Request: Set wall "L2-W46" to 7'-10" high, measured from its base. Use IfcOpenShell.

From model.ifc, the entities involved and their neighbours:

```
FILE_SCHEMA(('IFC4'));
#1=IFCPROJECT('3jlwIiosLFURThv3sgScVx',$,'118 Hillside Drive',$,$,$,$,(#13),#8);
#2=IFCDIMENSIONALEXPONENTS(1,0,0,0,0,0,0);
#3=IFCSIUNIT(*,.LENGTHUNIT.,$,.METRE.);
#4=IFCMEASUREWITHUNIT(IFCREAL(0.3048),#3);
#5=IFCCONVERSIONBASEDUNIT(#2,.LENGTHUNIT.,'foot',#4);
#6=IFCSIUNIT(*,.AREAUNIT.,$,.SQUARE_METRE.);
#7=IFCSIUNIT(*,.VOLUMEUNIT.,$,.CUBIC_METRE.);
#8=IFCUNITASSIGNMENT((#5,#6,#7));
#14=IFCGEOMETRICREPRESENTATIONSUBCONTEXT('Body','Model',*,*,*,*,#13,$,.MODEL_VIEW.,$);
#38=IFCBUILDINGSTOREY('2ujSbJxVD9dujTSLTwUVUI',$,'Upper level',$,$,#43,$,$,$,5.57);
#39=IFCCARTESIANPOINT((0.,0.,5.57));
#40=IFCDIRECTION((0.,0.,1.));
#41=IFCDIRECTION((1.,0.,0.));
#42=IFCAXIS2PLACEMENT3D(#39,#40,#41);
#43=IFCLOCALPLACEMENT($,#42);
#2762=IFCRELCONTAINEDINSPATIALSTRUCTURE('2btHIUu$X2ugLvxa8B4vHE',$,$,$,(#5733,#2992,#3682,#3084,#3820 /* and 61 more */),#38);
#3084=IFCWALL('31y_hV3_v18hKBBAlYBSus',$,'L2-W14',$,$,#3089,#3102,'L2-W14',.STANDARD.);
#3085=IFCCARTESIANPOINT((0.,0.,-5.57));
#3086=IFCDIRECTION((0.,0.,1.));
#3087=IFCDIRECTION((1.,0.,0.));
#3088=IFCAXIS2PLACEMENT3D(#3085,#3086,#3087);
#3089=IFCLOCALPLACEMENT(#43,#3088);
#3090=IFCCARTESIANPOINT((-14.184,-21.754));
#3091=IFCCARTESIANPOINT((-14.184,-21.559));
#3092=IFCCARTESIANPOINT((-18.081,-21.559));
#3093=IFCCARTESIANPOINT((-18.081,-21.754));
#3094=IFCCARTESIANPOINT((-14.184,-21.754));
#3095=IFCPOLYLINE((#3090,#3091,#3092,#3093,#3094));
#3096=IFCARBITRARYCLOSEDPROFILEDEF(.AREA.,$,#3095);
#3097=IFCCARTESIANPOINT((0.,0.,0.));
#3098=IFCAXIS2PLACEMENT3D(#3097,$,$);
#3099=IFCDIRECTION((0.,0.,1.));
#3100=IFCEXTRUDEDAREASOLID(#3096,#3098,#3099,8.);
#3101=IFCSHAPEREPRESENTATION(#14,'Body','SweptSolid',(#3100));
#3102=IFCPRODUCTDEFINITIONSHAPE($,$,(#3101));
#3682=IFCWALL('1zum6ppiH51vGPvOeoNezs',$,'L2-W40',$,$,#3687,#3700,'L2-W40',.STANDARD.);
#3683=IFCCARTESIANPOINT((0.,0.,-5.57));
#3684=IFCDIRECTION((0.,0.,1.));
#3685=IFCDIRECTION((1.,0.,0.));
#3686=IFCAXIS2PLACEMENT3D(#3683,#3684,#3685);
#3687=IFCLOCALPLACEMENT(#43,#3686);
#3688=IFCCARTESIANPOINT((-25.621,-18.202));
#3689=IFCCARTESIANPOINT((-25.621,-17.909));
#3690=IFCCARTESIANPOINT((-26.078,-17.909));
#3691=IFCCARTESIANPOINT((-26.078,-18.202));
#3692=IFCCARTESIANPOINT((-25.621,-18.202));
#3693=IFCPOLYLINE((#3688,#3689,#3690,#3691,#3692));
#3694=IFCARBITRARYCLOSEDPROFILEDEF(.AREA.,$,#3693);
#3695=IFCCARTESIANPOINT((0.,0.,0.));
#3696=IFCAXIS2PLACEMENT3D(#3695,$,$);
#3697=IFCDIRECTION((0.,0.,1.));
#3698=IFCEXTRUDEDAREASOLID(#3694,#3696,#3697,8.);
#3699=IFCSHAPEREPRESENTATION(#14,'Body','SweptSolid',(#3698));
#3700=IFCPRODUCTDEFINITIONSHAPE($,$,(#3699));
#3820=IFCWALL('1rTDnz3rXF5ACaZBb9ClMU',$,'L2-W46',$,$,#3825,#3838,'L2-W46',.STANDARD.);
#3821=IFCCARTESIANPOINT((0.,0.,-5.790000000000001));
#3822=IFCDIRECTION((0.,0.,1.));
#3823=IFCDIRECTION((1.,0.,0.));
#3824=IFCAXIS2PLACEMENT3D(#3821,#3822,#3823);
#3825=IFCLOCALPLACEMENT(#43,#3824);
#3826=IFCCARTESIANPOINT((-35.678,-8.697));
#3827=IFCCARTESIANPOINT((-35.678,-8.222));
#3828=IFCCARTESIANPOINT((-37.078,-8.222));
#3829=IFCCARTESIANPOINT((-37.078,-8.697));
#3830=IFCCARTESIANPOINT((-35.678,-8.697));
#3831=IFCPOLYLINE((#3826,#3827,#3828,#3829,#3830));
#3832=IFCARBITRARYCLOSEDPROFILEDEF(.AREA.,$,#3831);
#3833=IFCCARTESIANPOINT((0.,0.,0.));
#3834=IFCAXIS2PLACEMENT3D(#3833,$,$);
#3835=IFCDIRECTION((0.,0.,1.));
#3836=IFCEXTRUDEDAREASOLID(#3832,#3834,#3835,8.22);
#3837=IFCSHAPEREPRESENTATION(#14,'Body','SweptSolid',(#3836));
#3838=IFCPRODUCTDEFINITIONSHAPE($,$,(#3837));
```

```python
import ifcopenshell
import ifcopenshell.geom
import ifcopenshell.util.representation
import ifcopenshell.util.shape
import ifcopenshell.util.unit

model = ifcopenshell.open("model.ifc")
unit_scale = ifcopenshell.util.unit.calculate_unit_scale(model)
settings = ifcopenshell.geom.settings()


def volume(element):
    """Net volume in cubic metres, openings subtracted."""
    shape = ifcopenshell.geom.create_shape(settings, element)
    return ifcopenshell.util.shape.get_volume(shape.geometry)


wall = model.by_guid("1rTDnz3rXF5ACaZBb9ClMU")
before = volume(wall)

body = ifcopenshell.util.representation.get_representation(wall, "Model", "Body")
solid = body.Items[0]
old_height = solid.Depth
solid.Depth = 94 * 0.0254 / unit_scale
after = volume(wall)

print(f"height {old_height:g} -> {solid.Depth:g}, volume {before:.3f} -> {after:.3f} m3")

model.write("model_rev.ifc")
```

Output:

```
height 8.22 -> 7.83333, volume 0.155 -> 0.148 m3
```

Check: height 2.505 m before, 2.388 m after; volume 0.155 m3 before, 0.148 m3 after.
